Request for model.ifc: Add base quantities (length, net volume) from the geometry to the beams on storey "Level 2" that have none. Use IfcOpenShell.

First a look at what the model holds.

```python
import ifcopenshell
import ifcopenshell.util.element
import ifcopenshell.util.unit

model = ifcopenshell.open("model.ifc")
print(model.schema)
for unit_type in ("LENGTHUNIT", "AREAUNIT", "VOLUMEUNIT"):
    print(unit_type, ifcopenshell.util.unit.calculate_unit_scale(model, unit_type))
storey = next(s for s in model.by_type("IfcBuildingStorey") if s.Name == "Level 2")
beams = [e for e in ifcopenshell.util.element.get_decomposition(storey) if e.is_a("IfcBeam")]
for e in sorted(beams, key=lambda e: e.id()):
    print(e.id(), e.is_a(), e.Name, list(ifcopenshell.util.element.get_psets(e, qtos_only=True)), sep=" | ")
```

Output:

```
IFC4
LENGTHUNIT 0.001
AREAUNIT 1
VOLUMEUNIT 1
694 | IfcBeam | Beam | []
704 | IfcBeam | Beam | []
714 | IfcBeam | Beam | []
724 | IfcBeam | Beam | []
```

```python
import ifcopenshell
import ifcopenshell.api.pset
import ifcopenshell.geom
import ifcopenshell.util.element
import ifcopenshell.util.shape
import ifcopenshell.util.unit

model = ifcopenshell.open("model.ifc")
unit_scale = ifcopenshell.util.unit.calculate_unit_scale(model)
volume_scale = ifcopenshell.util.unit.calculate_unit_scale(model, "VOLUMEUNIT")
settings = ifcopenshell.geom.settings()

storey = next(s for s in model.by_type("IfcBuildingStorey") if s.Name == "Level 2")
beams = [e for e in ifcopenshell.util.element.get_decomposition(storey) if e.is_a("IfcBeam")]

for e in sorted(beams, key=lambda e: e.id()):
    if ifcopenshell.util.element.get_psets(e, qtos_only=True, should_inherit=False):
        continue
    # Geometry comes back in metres, in the element's own axes.
    shape = ifcopenshell.geom.create_shape(settings, e)
    values = {
        "Length": ifcopenshell.util.shape.get_max_xyz(shape.geometry) / unit_scale,
        "NetVolume": ifcopenshell.util.shape.get_volume(shape.geometry) / volume_scale,
    }
    qto = ifcopenshell.api.pset.add_qto(model, product=e, name="Qto_BeamBaseQuantities")
    ifcopenshell.api.pset.edit_qto(model, qto=qto, properties=values)
    print(e.id(), {k: round(v, 3) for k, v in values.items()})

model.write("model_rev.ifc")
```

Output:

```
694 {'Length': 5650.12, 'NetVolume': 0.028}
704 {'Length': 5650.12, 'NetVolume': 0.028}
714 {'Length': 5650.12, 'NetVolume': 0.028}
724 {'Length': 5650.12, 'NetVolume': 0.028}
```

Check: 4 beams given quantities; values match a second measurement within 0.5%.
